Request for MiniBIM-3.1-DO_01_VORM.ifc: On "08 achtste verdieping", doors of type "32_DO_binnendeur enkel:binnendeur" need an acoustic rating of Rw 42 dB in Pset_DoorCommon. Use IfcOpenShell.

First a look at what the model holds.

```python
import ifcopenshell
import ifcopenshell.util.element

model = ifcopenshell.open("MiniBIM-3.1-DO_01_VORM.ifc")
print(model.schema)
storey = next(s for s in model.by_type("IfcBuildingStorey") if s.Name == "08 achtste verdieping")
doors = [e for e in ifcopenshell.util.element.get_decomposition(storey) if e.is_a("IfcDoor")]
seen = {}
for e in doors:
    element_type = ifcopenshell.util.element.get_type(e)
    key = (element_type.Name if element_type != e and element_type else None, ifcopenshell.util.element.get_pset(e, "Pset_DoorCommon", "AcousticRating"))
    seen[key] = seen.get(key, 0) + 1
for (name, value), count in sorted(seen.items(), key=str):
    print(count, "x", name, "|", value)
```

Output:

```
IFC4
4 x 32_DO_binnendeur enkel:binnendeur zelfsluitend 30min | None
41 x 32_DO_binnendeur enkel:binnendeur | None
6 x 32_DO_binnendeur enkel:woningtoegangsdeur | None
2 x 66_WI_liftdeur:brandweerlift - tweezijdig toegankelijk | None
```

```python
import ifcopenshell
import ifcopenshell.api.pset
import ifcopenshell.util.element

model = ifcopenshell.open("MiniBIM-3.1-DO_01_VORM.ifc")

storey = next(s for s in model.by_type("IfcBuildingStorey") if s.Name == "08 achtste verdieping")
doors = [e for e in ifcopenshell.util.element.get_decomposition(storey) if e.is_a("IfcDoor")]

count = 0
for e in doors:
    element_type = ifcopenshell.util.element.get_type(e)
    if element_type in (None, e) or element_type.Name != "32_DO_binnendeur enkel:binnendeur":
        continue
    # add_pset returns the element's existing set when there is one.
    pset = ifcopenshell.api.pset.add_pset(model, product=e, name="Pset_DoorCommon")
    ifcopenshell.api.pset.edit_pset(model, pset=pset, properties={"AcousticRating": "Rw 42 dB"})
    count += 1

print(count, "doors updated")

model.write("MiniBIM-3.1-DO_01_VORM-out.ifc")
```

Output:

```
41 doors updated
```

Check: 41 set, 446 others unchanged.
